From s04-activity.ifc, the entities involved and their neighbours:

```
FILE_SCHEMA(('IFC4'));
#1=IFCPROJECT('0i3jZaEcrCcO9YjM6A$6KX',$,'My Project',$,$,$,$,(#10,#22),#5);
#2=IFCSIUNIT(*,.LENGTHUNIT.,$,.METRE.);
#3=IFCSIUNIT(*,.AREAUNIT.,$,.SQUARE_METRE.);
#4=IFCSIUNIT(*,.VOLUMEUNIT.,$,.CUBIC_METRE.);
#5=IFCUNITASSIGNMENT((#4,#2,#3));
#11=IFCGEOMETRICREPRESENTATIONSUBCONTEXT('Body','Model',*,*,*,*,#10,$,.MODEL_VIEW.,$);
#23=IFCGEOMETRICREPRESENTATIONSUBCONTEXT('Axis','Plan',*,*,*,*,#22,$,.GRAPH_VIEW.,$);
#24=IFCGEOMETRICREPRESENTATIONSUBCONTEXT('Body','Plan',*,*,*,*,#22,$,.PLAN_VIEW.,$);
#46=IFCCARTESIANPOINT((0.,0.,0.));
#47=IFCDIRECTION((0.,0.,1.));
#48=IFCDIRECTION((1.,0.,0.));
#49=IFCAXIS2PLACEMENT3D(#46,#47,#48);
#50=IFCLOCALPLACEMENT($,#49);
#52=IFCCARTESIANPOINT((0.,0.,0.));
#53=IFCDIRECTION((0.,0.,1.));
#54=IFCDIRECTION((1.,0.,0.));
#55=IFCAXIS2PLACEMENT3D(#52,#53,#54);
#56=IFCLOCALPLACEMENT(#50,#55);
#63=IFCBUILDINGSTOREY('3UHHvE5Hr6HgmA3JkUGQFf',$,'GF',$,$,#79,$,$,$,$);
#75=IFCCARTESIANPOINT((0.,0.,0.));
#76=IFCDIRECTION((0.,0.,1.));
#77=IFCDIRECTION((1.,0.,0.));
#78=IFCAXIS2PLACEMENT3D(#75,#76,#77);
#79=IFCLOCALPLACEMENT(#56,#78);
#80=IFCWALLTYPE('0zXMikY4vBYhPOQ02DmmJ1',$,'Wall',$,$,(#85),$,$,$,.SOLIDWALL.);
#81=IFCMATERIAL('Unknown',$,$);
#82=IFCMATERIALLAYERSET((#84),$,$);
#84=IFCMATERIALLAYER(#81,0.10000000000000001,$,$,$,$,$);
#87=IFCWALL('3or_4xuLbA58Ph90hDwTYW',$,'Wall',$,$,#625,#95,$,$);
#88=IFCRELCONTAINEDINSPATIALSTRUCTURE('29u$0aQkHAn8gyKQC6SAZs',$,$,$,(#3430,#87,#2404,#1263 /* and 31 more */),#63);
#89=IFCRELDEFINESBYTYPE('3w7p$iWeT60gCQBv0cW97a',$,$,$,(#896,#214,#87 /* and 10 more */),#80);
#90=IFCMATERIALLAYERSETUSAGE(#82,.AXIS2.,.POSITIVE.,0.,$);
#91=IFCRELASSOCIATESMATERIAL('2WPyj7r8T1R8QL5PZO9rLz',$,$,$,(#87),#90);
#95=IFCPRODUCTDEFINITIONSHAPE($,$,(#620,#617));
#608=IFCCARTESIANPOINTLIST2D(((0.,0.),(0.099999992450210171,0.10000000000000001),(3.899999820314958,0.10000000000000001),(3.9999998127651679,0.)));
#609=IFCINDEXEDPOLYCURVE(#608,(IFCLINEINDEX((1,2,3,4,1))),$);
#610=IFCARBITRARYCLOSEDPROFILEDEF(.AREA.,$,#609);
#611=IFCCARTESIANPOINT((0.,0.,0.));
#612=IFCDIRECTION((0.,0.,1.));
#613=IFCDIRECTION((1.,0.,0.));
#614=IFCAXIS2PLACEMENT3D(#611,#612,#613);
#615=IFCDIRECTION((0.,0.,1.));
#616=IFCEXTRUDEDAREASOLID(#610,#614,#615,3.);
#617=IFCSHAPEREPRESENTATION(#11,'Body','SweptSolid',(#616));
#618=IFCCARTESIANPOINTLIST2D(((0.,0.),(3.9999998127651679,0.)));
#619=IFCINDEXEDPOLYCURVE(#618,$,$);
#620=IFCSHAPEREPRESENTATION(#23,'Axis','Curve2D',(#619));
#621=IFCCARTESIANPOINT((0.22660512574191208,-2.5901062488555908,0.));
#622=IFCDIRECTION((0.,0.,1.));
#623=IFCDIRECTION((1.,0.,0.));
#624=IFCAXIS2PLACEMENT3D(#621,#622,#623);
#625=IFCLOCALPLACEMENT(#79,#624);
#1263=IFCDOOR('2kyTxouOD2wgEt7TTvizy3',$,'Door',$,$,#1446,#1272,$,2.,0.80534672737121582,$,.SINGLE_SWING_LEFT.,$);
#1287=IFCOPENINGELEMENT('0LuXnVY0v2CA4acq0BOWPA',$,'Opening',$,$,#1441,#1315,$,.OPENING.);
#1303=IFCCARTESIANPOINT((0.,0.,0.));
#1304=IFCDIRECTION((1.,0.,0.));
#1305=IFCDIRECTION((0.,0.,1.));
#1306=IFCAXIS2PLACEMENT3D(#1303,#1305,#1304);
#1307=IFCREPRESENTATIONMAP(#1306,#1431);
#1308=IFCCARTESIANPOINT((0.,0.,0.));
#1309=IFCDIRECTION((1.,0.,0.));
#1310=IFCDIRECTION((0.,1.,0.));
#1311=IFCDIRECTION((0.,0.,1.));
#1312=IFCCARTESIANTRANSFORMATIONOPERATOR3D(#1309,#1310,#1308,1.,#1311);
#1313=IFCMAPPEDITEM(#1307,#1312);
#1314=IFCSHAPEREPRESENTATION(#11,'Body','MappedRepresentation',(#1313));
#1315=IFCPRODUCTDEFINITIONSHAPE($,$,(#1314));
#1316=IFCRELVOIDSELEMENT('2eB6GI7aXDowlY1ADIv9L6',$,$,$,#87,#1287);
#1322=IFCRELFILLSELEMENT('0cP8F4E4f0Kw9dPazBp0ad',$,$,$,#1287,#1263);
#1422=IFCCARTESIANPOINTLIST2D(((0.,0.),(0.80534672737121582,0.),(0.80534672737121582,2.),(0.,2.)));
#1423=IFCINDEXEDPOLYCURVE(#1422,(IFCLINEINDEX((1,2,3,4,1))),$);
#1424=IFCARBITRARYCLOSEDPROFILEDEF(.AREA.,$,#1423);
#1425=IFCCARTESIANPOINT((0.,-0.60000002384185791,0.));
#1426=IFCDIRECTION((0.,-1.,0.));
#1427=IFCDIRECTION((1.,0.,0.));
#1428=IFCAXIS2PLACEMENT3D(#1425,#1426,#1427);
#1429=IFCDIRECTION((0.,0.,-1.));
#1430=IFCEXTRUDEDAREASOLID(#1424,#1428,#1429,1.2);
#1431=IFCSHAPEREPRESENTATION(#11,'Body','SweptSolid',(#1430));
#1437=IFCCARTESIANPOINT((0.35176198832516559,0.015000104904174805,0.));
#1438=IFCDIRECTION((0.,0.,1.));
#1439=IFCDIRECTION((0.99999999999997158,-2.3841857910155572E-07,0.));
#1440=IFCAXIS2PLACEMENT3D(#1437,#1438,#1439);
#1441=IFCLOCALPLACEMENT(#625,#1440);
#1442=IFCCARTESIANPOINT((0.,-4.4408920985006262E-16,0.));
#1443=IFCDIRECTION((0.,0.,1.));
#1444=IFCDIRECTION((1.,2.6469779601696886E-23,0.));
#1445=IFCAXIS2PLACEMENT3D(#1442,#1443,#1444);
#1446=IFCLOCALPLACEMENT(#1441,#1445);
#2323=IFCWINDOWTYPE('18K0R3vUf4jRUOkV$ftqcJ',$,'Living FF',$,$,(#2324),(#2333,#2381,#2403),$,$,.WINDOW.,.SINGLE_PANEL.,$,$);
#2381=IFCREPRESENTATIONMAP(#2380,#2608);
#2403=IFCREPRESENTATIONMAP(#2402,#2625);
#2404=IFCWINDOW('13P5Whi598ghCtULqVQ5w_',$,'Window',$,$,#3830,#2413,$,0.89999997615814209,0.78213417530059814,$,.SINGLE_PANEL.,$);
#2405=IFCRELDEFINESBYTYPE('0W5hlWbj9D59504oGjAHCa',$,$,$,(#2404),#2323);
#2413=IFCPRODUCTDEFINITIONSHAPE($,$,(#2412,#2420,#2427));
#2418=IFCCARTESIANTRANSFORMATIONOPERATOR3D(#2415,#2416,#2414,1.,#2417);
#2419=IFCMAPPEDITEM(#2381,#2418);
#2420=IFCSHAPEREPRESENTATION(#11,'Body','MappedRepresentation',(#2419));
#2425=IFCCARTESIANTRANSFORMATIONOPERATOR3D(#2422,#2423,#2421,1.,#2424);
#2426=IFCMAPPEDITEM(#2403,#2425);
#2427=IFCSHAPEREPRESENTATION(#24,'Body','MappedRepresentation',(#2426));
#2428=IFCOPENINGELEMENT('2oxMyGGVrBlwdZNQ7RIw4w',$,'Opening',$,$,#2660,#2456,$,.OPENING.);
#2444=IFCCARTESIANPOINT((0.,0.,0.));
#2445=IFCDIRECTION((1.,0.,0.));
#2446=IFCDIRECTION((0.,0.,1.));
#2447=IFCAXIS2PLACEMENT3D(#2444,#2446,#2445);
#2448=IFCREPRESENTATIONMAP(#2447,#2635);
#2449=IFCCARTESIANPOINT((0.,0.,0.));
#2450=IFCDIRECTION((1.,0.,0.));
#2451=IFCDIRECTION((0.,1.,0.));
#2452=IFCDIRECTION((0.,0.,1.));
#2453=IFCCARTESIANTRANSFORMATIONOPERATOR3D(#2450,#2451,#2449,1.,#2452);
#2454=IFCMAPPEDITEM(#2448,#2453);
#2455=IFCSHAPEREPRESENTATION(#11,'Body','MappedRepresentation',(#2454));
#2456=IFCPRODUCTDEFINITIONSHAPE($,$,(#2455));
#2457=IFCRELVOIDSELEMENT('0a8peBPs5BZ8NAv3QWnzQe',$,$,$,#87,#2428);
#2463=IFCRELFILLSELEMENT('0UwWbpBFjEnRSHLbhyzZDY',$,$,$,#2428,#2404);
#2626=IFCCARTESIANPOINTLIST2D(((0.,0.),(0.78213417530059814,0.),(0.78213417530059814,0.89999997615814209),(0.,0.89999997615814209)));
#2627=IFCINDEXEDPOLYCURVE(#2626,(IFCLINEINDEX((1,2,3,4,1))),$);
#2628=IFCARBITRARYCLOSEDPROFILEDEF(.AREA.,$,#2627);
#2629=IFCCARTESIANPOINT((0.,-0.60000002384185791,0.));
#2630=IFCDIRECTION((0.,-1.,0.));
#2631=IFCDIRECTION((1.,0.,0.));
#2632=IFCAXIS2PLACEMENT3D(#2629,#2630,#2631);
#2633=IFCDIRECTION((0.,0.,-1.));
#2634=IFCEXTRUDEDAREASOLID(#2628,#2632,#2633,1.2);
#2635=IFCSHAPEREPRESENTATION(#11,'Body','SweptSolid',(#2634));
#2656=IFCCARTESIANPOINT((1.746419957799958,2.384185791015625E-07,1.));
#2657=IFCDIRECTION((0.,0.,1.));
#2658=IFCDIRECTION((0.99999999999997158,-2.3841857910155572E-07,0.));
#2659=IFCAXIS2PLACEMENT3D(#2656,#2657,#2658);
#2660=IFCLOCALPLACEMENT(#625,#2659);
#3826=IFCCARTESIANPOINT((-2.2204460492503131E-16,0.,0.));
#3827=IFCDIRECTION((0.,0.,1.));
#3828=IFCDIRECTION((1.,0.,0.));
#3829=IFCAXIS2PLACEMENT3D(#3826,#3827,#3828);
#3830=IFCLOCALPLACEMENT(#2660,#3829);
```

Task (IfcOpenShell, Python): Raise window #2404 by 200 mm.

```python
import numpy as np
import ifcopenshell
import ifcopenshell.api.geometry
import ifcopenshell.util.placement
import ifcopenshell.util.unit

model = ifcopenshell.open("s04-activity.ifc")
unit_scale = ifcopenshell.util.unit.calculate_unit_scale(model)

window = model.by_id(2404)
opening = window.FillsVoids[0].RelatingOpeningElement
dz = 0.2

shift = np.array([0.0, 0.0, dz])
# The window is placed relative to its opening, so it follows when the opening moves.
matrix = ifcopenshell.util.placement.get_local_placement(opening.ObjectPlacement)
matrix[:3, 3] += shift
ifcopenshell.api.geometry.edit_object_placement(
    model, product=opening, matrix=matrix, is_si=False, should_transform_children=True
)

print(f"moved by {dz * unit_scale:+.3f} m")

model.write("s04-activity-out.ifc")
```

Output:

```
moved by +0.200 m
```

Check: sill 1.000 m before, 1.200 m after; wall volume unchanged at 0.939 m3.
